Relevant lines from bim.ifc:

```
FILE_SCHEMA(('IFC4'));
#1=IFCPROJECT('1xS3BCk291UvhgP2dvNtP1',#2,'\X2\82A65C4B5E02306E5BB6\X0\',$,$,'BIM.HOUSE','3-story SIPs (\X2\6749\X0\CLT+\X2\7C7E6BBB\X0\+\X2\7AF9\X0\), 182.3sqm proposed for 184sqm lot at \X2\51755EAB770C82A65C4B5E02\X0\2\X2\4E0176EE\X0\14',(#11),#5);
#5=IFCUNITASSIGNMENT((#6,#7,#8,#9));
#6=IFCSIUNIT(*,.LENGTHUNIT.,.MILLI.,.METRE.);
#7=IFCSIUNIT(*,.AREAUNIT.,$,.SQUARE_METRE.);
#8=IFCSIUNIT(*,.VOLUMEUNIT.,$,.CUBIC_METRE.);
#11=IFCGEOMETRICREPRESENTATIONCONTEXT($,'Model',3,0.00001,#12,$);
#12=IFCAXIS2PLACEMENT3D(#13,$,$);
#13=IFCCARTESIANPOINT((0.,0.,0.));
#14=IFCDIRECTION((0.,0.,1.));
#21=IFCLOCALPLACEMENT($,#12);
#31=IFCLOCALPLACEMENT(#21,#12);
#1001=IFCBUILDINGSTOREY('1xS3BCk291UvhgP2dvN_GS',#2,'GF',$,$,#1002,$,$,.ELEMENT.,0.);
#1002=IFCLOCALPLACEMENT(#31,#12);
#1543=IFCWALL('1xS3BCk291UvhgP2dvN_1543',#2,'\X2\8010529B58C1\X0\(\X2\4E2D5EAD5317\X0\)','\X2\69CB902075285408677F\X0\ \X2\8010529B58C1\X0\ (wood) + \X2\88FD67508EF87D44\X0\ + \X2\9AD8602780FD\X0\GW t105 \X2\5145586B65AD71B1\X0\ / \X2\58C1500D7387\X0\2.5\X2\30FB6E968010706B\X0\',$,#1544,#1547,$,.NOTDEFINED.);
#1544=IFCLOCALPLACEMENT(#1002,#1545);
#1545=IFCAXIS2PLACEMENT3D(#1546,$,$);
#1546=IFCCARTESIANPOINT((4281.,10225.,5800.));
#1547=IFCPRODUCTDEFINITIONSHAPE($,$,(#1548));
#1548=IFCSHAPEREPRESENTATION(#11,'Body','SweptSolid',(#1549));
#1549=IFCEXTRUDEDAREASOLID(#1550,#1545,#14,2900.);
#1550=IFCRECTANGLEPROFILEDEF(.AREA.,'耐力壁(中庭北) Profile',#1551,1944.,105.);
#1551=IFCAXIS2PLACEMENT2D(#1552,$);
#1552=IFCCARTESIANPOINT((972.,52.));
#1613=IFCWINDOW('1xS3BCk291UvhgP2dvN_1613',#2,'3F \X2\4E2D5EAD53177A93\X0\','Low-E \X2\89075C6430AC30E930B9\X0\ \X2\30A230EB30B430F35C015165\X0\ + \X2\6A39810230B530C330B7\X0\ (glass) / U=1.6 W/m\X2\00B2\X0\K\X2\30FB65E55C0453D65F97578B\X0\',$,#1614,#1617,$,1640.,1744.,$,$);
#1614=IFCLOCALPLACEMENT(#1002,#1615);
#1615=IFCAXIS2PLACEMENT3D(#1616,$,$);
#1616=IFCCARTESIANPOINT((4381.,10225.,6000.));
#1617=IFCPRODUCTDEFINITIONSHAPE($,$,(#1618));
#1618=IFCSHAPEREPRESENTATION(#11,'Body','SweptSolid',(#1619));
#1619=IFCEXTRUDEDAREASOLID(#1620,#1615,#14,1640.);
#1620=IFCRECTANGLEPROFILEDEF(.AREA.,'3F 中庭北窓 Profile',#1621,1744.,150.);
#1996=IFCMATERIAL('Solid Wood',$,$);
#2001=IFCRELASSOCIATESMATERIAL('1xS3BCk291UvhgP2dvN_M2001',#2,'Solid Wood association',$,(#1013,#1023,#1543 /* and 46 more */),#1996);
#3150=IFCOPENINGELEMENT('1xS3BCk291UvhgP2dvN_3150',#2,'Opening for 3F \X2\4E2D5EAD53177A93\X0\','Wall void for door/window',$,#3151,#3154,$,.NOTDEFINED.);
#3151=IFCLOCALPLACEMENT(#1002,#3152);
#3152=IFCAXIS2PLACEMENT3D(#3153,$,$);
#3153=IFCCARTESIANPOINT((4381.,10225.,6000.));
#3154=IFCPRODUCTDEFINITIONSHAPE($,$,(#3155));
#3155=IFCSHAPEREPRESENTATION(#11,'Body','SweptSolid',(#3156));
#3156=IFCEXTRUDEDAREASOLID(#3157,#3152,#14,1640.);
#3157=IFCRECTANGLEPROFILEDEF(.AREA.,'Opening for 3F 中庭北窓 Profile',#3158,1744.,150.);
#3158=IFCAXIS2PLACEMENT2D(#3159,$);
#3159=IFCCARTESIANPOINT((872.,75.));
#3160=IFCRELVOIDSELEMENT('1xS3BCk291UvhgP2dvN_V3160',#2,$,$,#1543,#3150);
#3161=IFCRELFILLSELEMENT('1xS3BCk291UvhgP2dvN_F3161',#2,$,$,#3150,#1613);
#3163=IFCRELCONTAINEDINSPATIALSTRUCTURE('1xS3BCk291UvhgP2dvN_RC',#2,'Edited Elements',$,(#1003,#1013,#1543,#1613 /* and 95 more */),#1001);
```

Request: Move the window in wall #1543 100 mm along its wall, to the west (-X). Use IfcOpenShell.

```python
import ifcopenshell
import ifcopenshell.api.geometry
import ifcopenshell.util.placement
import ifcopenshell.util.unit

model = ifcopenshell.open("bim.ifc")
unit_scale = ifcopenshell.util.unit.calculate_unit_scale(model)

window = model.by_id(1613)
opening = window.FillsVoids[0].RelatingOpeningElement
wall = opening.VoidsElements[0].RelatingBuildingElement

wall_matrix = ifcopenshell.util.placement.get_local_placement(wall.ObjectPlacement)
shift = wall_matrix[:3, 0] * -0.1 / unit_scale
before = ifcopenshell.util.placement.get_local_placement(window.ObjectPlacement)[:3, 3].copy()

# The window is not placed relative to its opening, so move both.
for product in (opening, window):
    matrix = ifcopenshell.util.placement.get_local_placement(product.ObjectPlacement)
    matrix[:3, 3] += shift
    ifcopenshell.api.geometry.edit_object_placement(model, product=product, matrix=matrix, is_si=False)

after = ifcopenshell.util.placement.get_local_placement(window.ObjectPlacement)[:3, 3]
print("window moved by", (after - before).round(3) + 0.0)

model.write("bim-out.ifc")
```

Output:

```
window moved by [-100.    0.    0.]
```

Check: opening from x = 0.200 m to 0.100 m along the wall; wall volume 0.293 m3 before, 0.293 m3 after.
